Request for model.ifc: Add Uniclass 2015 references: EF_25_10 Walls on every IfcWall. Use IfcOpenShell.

First a look at what the model holds.

```python
import ifcopenshell

model = ifcopenshell.open("model.ifc")
print(model.schema)
print("classifications:", [c.Name for c in model.by_type("IfcClassification")])
for ifc_class in ("IfcDoor", "IfcRoof", "IfcStair", "IfcWall", "IfcWindow"):
    print(ifc_class, len(model.by_type(ifc_class)))
```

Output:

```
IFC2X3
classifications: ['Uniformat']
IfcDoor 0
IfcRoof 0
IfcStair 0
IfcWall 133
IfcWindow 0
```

```python
import ifcopenshell
import ifcopenshell.api.classification

model = ifcopenshell.open("model.ifc")

# IFC2X3 requires Source and Edition and has no link from the project to the system.
system = model.create_entity("IfcClassification", Source="NBS", Edition="2015", Name="Uniclass 2015")

codes = {
    "IfcWall": ("EF_25_10", "Walls"),
}
for ifc_class, (code, name) in codes.items():
    products = model.by_type(ifc_class)
    ifcopenshell.api.classification.add_reference(
        model, products=products, classification=system, identification=code, name=name
    )
    print(code, len(products))

model.write("model-out.ifc")
```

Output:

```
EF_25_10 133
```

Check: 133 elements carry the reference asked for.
